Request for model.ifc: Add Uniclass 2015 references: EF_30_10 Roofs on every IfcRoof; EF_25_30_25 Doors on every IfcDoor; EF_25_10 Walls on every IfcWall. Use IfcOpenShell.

First a look at what the model holds.

```python
import ifcopenshell

model = ifcopenshell.open("model.ifc")
print(model.schema)
print("classifications:", [c.Name for c in model.by_type("IfcClassification")])
for ifc_class in ("IfcDoor", "IfcRoof", "IfcStair", "IfcWall", "IfcWindow"):
    print(ifc_class, len(model.by_type(ifc_class)))
```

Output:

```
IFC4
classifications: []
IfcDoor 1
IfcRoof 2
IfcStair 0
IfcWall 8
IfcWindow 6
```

```python
import ifcopenshell
import ifcopenshell.api.classification

model = ifcopenshell.open("model.ifc")

system = ifcopenshell.api.classification.add_classification(model, classification="Uniclass 2015")

codes = {
    "IfcRoof": ("EF_30_10", "Roofs"),
    "IfcDoor": ("EF_25_30_25", "Doors"),
    "IfcWall": ("EF_25_10", "Walls"),
}
for ifc_class, (code, name) in codes.items():
    products = model.by_type(ifc_class)
    ifcopenshell.api.classification.add_reference(
        model, products=products, classification=system, identification=code, name=name
    )
    print(code, len(products))

model.write("model_v2.ifc")
```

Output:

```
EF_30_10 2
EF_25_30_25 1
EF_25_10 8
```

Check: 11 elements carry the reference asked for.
